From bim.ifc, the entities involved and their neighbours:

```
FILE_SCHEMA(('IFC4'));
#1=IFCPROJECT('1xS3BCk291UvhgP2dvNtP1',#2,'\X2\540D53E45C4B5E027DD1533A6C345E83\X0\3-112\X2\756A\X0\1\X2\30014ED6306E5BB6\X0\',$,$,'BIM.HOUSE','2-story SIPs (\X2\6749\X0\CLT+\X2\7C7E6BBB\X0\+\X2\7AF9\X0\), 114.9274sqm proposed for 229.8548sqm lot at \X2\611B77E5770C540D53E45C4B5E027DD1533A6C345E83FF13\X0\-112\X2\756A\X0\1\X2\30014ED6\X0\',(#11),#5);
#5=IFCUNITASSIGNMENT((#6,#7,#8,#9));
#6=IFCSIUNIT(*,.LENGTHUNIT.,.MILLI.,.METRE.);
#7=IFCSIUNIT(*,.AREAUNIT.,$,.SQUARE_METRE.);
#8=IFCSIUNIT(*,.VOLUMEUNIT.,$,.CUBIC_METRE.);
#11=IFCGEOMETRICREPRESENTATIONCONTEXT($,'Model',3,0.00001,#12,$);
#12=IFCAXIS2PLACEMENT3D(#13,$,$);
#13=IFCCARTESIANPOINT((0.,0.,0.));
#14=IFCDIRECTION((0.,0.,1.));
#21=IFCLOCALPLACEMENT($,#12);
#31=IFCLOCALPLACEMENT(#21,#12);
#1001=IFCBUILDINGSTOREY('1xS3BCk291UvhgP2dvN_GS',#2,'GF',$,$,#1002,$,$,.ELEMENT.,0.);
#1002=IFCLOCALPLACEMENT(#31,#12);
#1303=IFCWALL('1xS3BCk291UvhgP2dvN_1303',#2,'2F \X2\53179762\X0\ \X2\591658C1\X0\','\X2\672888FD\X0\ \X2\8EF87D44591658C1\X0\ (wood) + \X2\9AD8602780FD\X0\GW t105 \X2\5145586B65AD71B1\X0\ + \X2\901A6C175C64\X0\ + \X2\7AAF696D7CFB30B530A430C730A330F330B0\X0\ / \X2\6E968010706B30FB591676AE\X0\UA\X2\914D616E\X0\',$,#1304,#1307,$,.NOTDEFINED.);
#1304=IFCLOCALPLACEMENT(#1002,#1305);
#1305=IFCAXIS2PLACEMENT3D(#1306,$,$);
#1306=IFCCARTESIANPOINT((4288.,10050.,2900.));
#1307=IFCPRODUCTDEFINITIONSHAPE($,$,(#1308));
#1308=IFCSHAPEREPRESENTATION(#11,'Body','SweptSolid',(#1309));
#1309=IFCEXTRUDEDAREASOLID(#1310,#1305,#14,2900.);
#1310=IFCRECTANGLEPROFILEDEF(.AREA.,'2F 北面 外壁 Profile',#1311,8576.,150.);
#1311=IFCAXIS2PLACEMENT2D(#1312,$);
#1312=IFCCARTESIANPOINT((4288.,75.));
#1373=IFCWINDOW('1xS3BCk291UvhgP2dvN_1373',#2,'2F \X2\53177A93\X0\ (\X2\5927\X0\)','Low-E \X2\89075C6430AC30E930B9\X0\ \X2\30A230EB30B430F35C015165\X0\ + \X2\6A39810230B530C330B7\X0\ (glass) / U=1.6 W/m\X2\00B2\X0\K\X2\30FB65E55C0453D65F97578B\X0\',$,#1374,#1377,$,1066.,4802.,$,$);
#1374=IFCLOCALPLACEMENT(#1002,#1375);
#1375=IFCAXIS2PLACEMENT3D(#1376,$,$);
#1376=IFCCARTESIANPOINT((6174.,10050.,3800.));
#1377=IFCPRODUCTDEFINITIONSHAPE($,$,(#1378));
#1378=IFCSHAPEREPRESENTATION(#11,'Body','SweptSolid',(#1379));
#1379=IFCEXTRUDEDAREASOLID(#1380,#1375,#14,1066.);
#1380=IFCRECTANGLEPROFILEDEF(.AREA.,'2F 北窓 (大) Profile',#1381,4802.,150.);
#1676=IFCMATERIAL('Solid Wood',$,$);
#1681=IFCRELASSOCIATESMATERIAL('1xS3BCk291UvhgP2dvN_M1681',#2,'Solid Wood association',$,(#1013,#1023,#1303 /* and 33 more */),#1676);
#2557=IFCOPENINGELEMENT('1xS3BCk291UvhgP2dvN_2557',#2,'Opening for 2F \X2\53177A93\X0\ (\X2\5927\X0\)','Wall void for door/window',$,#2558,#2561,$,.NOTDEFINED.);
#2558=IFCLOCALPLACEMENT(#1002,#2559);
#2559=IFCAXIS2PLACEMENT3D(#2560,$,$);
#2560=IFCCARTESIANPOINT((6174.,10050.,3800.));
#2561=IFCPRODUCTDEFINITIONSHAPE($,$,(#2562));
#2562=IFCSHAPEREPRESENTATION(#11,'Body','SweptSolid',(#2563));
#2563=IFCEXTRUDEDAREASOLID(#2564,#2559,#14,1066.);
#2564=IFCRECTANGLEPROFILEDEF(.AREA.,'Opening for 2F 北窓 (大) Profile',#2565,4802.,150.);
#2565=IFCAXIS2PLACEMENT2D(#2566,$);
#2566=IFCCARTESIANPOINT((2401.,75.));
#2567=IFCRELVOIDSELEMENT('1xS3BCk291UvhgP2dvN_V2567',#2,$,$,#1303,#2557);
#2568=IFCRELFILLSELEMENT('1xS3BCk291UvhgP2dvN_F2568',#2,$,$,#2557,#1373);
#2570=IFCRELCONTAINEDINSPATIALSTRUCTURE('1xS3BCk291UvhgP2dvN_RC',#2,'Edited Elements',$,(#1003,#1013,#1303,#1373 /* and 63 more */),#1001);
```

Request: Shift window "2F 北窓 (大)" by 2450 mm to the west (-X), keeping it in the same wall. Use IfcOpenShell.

```python
import ifcopenshell
import ifcopenshell.api.geometry
import ifcopenshell.util.placement
import ifcopenshell.util.unit

model = ifcopenshell.open("bim.ifc")
unit_scale = ifcopenshell.util.unit.calculate_unit_scale(model)

window = model.by_guid("1xS3BCk291UvhgP2dvN_1373")
opening = window.FillsVoids[0].RelatingOpeningElement
wall = opening.VoidsElements[0].RelatingBuildingElement

wall_matrix = ifcopenshell.util.placement.get_local_placement(wall.ObjectPlacement)
shift = wall_matrix[:3, 0] * -2.45 / unit_scale
before = ifcopenshell.util.placement.get_local_placement(window.ObjectPlacement)[:3, 3].copy()

# The window is not placed relative to its opening, so move both.
for product in (opening, window):
    matrix = ifcopenshell.util.placement.get_local_placement(product.ObjectPlacement)
    matrix[:3, 3] += shift
    ifcopenshell.api.geometry.edit_object_placement(model, product=product, matrix=matrix, is_si=False)

after = ifcopenshell.util.placement.get_local_placement(window.ObjectPlacement)[:3, 3]
print("window moved by", (after - before).round(3) + 0.0)

model.write("bim_edited.ifc")
```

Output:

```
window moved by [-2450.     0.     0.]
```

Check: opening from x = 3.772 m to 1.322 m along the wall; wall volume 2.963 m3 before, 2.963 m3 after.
